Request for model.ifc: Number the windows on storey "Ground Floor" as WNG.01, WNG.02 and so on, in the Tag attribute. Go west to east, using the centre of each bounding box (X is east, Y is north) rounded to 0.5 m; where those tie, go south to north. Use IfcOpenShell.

First a look at what the model holds.

```python
import ifcopenshell
import ifcopenshell.util.element
import ifcopenshell.util.placement

model = ifcopenshell.open("model.ifc")
print(model.schema)
storey = next(s for s in model.by_type("IfcBuildingStorey") if s.Name == "Ground Floor")
windows = [e for e in ifcopenshell.util.element.get_decomposition(storey) if e.is_a("IfcWindow")]
for e in sorted(windows, key=lambda e: e.id()):
    origin = ifcopenshell.util.placement.get_local_placement(e.ObjectPlacement)[:3, 3]
    print(e.id(), e.Tag, e.Name, origin.round(2) + 0.0, sep=" | ")
```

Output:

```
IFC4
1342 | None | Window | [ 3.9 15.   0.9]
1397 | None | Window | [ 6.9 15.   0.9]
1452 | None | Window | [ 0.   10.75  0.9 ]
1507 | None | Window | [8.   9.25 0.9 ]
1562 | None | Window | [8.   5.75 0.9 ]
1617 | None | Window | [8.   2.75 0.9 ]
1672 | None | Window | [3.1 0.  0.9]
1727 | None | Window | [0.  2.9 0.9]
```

```python
import ifcopenshell
import ifcopenshell.geom
import ifcopenshell.util.element
import ifcopenshell.util.shape

model = ifcopenshell.open("model.ifc")
settings = ifcopenshell.geom.settings()
settings.set("use-world-coords", True)


def centre(element):
    shape = ifcopenshell.geom.create_shape(settings, element)
    return ifcopenshell.util.shape.get_bbox_centroid(shape.geometry)


storey = next(s for s in model.by_type("IfcBuildingStorey") if s.Name == "Ground Floor")
windows = [e for e in ifcopenshell.util.element.get_decomposition(storey) if e.is_a("IfcWindow")]

# Insertion points can sit at a corner or the storey origin, so sort by the geometry (in metres).
centres = {e: centre(e) for e in windows}
windows.sort(key=lambda e: (round(centres[e][0] / 0.5), centres[e][1]))

for i, e in enumerate(windows, start=1):
    number = f"WNG.{i:02d}"
    e.Tag = number
    print(e.id(), number)

model.write("model_edited.ifc")
```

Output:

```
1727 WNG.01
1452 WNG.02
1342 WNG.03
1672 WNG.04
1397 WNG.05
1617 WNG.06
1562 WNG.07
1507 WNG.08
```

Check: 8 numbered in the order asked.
